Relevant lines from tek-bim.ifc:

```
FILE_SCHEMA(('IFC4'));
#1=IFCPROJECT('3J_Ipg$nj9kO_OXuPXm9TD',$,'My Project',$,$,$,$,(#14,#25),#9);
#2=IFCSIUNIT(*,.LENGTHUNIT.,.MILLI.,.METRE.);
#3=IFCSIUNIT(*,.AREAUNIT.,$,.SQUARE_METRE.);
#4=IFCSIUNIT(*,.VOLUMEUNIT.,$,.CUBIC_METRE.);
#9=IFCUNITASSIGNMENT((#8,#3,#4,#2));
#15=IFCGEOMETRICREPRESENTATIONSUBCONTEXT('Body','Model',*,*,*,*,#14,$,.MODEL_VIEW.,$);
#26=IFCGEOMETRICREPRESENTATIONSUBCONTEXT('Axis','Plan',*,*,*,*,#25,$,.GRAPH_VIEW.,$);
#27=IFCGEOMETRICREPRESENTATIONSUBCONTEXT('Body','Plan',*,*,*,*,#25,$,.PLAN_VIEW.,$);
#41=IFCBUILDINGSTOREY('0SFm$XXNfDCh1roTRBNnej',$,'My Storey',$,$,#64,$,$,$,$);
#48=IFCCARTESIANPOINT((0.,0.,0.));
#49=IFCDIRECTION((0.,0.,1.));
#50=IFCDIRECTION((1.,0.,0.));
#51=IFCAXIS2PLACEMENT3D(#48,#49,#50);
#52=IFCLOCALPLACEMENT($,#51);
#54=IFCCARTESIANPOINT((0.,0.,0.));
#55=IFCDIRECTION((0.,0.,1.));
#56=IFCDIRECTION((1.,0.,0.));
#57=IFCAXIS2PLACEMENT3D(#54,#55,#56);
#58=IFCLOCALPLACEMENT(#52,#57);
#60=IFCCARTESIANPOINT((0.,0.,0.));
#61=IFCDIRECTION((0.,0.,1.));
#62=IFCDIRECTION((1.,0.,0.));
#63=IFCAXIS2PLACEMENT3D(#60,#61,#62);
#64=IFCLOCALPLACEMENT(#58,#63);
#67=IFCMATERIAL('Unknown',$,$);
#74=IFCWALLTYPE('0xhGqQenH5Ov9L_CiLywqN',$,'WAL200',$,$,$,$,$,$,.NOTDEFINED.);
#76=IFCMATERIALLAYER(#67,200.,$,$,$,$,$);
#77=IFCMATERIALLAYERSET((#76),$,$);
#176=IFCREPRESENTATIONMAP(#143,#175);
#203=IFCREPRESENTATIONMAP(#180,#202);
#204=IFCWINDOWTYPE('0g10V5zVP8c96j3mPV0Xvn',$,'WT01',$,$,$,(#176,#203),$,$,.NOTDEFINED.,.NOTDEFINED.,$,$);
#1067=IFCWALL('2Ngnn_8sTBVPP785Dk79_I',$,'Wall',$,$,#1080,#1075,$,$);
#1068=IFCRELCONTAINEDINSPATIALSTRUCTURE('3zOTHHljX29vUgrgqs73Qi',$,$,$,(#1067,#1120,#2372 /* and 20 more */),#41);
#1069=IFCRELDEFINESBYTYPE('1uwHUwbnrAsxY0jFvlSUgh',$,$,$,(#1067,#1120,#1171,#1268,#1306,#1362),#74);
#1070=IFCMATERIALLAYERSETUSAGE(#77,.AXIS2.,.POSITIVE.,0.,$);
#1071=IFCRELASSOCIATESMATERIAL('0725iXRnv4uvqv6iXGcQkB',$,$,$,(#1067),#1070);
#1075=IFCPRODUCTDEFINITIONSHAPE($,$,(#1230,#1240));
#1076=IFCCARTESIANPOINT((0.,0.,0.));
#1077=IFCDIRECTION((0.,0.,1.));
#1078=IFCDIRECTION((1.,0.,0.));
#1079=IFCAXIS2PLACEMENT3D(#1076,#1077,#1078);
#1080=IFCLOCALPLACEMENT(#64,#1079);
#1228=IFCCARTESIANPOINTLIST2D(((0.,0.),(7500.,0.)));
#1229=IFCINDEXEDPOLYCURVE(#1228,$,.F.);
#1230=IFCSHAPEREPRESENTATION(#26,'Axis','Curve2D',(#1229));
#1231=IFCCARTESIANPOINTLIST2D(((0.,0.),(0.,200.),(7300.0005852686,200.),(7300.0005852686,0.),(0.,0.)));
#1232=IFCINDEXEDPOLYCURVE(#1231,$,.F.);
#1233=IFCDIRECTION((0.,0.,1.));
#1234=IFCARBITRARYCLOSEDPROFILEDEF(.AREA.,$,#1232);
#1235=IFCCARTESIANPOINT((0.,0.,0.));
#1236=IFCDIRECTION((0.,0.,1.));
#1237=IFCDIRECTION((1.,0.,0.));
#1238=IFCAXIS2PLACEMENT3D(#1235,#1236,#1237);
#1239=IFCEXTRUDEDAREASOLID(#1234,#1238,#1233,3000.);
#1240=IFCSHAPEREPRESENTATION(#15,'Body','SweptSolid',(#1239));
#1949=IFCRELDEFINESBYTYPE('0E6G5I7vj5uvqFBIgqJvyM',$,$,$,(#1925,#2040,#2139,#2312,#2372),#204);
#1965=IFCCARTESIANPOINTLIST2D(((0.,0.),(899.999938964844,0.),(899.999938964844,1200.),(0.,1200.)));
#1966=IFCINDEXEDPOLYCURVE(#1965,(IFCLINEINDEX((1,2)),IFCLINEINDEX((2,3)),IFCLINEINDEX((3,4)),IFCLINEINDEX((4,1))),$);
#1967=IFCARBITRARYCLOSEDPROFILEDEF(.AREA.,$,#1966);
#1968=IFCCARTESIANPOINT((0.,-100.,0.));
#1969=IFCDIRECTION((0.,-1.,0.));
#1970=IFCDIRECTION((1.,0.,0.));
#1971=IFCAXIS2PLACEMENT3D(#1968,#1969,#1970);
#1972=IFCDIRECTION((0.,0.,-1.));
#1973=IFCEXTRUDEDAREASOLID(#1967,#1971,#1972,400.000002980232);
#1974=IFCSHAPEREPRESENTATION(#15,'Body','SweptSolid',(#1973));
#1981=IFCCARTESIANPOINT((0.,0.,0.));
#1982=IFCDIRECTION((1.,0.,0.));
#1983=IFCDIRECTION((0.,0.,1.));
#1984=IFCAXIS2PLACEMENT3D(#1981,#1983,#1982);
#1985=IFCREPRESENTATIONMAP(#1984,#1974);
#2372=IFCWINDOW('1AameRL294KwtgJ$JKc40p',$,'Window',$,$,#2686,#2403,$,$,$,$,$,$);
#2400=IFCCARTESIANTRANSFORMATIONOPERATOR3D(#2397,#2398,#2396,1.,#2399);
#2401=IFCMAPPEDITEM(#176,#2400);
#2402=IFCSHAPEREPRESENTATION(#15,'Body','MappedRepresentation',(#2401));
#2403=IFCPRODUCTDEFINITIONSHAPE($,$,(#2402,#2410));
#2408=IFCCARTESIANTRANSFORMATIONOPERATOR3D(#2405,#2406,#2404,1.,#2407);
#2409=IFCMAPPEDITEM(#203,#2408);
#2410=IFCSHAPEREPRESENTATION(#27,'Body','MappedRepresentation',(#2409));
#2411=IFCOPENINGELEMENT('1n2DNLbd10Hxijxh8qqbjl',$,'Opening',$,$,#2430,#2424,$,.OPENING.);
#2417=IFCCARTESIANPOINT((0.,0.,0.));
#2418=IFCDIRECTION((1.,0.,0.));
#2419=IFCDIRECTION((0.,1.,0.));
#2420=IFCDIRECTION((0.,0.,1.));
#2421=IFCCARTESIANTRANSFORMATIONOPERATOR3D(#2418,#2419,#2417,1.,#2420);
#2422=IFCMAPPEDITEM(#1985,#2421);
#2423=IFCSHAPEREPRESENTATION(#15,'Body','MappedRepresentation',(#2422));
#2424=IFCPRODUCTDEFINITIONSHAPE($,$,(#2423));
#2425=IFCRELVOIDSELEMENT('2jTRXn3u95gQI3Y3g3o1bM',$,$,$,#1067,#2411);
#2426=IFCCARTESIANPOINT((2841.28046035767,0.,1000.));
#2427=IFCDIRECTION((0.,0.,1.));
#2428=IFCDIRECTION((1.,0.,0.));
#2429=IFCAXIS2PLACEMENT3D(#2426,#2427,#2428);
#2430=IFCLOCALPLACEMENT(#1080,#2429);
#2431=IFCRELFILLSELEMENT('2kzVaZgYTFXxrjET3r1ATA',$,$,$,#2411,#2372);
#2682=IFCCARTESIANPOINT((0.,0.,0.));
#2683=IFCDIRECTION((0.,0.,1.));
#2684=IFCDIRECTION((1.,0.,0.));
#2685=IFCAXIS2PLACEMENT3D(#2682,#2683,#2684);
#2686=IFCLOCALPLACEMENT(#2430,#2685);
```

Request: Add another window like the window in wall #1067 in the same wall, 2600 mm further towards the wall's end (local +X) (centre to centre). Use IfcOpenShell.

```python
import ifcopenshell
import ifcopenshell.api.feature
import ifcopenshell.api.geometry
import ifcopenshell.api.root
import ifcopenshell.geom
import ifcopenshell.util.element
import ifcopenshell.util.placement
import ifcopenshell.util.shape
import ifcopenshell.util.unit

model = ifcopenshell.open("tek-bim.ifc")
unit_scale = ifcopenshell.util.unit.calculate_unit_scale(model)
settings = ifcopenshell.geom.settings()


def volume(element):
    """Net volume in cubic metres, openings subtracted."""
    shape = ifcopenshell.geom.create_shape(settings, element)
    return ifcopenshell.util.shape.get_volume(shape.geometry)


window = model.by_guid("1AameRL294KwtgJ$JKc40p")
opening = window.FillsVoids[0].RelatingOpeningElement
wall = opening.VoidsElements[0].RelatingBuildingElement
before = volume(wall)
shift = ifcopenshell.util.placement.get_local_placement(wall.ObjectPlacement)[:3, 0] * 2.6 / unit_scale

# copy_class copies the void relationship, type, container and properties, but no geometry.
new_opening = ifcopenshell.api.root.copy_class(model, product=opening)
new_opening.Representation = ifcopenshell.util.element.copy_deep(
    model, opening.Representation, exclude=["IfcGeometricRepresentationContext", "IfcRepresentationMap"]
)
new_window = ifcopenshell.api.root.copy_class(model, product=window)
new_window.Representation = ifcopenshell.util.element.copy_deep(
    model, window.Representation, exclude=["IfcGeometricRepresentationContext", "IfcRepresentationMap"]
)
ifcopenshell.api.feature.add_filling(model, opening=new_opening, element=new_window)

for old, new in ((opening, new_opening), (window, new_window)):
    matrix = ifcopenshell.util.placement.get_local_placement(old.ObjectPlacement)
    matrix[:3, 3] += shift
    ifcopenshell.api.geometry.edit_object_placement(model, product=new, matrix=matrix, is_si=False)

after = volume(wall)

print(f"wall volume {before:.3f} -> {after:.3f} m3")

model.write("tek-bim_rev.ifc")
```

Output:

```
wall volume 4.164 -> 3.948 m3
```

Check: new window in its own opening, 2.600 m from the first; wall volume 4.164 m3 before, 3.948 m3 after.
